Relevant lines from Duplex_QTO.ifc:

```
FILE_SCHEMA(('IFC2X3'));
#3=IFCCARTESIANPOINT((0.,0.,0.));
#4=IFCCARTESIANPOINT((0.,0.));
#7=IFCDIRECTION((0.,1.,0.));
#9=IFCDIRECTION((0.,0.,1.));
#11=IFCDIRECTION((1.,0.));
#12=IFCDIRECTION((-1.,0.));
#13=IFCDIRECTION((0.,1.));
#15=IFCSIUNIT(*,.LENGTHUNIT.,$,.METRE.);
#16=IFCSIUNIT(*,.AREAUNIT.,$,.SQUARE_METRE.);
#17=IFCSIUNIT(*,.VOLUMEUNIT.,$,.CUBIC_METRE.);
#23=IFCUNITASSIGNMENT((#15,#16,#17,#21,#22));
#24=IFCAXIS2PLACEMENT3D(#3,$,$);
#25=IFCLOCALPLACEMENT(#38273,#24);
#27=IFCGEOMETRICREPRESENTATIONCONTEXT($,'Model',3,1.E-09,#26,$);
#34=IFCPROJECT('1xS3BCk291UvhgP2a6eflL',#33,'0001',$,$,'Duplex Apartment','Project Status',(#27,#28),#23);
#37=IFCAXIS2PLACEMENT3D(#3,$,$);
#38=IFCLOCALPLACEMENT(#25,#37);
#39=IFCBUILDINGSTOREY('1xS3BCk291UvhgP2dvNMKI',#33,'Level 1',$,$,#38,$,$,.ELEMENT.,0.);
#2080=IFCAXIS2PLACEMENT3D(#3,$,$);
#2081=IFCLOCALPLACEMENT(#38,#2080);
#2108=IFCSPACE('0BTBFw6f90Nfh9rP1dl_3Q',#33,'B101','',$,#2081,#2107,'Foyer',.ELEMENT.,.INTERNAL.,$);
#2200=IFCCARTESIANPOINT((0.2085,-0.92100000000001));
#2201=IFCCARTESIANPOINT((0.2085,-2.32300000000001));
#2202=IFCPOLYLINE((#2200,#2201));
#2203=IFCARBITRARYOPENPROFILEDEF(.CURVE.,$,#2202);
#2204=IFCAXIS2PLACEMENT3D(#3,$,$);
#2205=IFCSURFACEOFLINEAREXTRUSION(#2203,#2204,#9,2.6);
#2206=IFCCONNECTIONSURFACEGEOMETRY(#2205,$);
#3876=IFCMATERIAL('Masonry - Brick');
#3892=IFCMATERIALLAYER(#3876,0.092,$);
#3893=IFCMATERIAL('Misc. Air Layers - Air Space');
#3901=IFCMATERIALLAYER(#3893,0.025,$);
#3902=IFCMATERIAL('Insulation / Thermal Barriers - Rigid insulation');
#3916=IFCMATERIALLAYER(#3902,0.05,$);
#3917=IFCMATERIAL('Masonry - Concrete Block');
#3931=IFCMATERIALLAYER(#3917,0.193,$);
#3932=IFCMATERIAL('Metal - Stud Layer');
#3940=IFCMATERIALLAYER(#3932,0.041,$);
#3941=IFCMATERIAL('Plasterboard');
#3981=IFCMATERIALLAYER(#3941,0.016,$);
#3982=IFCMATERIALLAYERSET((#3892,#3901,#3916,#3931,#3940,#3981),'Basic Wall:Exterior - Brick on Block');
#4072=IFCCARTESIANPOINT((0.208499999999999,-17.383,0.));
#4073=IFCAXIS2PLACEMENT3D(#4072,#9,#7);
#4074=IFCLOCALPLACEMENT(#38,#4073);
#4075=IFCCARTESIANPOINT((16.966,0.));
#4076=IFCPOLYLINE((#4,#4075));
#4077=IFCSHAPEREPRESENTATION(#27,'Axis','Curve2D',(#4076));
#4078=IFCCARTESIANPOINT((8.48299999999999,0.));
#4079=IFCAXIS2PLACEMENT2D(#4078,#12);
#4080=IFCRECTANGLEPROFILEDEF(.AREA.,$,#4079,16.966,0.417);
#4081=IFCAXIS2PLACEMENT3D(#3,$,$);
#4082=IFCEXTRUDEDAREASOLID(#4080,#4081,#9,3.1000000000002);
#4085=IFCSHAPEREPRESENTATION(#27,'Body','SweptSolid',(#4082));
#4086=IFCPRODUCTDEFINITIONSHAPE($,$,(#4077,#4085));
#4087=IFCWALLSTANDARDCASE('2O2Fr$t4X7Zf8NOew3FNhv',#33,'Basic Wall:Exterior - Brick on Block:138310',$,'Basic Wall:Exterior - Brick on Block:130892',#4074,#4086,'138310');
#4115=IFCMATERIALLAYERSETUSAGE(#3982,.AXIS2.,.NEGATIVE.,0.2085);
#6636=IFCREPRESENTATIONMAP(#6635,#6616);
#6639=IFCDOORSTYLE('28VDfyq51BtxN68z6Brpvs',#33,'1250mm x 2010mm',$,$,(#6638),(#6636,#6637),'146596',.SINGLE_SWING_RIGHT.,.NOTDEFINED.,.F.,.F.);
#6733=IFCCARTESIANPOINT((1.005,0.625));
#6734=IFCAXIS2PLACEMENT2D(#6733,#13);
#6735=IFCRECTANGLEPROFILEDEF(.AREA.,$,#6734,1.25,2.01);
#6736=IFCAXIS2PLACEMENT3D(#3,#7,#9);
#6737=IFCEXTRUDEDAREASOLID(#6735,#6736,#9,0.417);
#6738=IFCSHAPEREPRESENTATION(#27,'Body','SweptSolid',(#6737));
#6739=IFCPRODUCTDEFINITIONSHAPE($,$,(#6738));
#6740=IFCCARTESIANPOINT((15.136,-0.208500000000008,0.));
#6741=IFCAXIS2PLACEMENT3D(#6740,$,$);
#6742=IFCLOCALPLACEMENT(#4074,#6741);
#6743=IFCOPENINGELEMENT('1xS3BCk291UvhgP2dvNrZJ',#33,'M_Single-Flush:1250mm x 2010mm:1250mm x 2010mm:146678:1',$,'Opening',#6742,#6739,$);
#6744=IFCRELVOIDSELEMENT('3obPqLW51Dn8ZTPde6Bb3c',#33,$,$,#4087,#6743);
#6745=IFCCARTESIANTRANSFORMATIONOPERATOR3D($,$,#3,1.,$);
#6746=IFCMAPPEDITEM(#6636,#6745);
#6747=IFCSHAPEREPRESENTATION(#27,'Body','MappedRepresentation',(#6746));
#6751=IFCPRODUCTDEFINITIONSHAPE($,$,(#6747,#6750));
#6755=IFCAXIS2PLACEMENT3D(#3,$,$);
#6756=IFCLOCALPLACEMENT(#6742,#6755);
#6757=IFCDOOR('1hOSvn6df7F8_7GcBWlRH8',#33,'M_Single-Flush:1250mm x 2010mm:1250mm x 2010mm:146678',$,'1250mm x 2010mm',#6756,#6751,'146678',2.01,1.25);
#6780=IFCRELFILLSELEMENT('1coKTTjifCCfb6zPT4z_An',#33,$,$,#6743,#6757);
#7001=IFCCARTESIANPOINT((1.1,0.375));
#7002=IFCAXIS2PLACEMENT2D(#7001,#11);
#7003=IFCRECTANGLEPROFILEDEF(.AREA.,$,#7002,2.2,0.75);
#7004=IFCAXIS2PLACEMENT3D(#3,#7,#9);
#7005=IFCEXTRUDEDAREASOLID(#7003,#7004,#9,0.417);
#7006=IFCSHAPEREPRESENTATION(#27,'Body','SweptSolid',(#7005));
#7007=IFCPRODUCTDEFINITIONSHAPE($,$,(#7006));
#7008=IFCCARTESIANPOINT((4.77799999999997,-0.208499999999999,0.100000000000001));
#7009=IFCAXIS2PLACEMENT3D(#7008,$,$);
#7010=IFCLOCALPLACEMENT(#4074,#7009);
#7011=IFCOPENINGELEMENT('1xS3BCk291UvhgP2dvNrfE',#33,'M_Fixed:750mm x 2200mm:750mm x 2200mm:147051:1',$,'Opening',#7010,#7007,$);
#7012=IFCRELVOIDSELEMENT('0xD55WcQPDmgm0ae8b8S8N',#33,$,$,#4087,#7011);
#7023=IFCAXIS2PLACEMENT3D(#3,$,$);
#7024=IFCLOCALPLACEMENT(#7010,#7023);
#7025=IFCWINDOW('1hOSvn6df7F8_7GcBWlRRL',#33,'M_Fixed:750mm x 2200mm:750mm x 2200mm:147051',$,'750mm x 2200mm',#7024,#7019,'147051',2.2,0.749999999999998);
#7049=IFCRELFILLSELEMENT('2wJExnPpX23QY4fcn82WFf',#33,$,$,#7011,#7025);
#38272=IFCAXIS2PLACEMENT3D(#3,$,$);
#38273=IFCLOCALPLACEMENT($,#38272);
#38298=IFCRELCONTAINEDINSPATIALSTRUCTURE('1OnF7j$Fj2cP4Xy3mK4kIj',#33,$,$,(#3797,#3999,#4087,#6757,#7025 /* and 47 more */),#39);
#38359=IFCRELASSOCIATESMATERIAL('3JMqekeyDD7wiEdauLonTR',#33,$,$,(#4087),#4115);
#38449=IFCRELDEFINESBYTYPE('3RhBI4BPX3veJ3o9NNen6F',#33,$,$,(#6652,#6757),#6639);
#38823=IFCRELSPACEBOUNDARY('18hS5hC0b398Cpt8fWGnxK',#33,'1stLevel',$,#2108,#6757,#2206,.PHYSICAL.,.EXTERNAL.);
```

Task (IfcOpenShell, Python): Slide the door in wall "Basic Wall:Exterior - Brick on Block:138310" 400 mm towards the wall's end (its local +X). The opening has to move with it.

```python
import numpy as np
import ifcopenshell
import ifcopenshell.api.geometry
import ifcopenshell.util.placement
import ifcopenshell.util.unit

model = ifcopenshell.open("Duplex_QTO.ifc")
unit_scale = ifcopenshell.util.unit.calculate_unit_scale(model)

door = model.by_guid("1hOSvn6df7F8_7GcBWlRH8")
opening = door.FillsVoids[0].RelatingOpeningElement
wall = opening.VoidsElements[0].RelatingBuildingElement

wall_matrix = ifcopenshell.util.placement.get_local_placement(wall.ObjectPlacement)
shift = wall_matrix[:3, 0] * 0.4 / unit_scale
before = ifcopenshell.util.placement.get_local_placement(door.ObjectPlacement)[:3, 3].copy()

# The door is placed relative to its opening, so it follows when the opening moves.
matrix = ifcopenshell.util.placement.get_local_placement(opening.ObjectPlacement)
matrix[:3, 3] += shift
ifcopenshell.api.geometry.edit_object_placement(
    model, product=opening, matrix=matrix, is_si=False, should_transform_children=True
)

# Space boundary surfaces are stored in each space's coordinates; move them too.
for rel in door.ProvidesBoundaries:
    if not rel.ConnectionGeometry:
        continue
    surface = rel.ConnectionGeometry.SurfaceOnRelatingElement
    space_matrix = ifcopenshell.util.placement.get_local_placement(rel.RelatingSpace.ObjectPlacement)
    point = np.array(surface.Position.Location.Coordinates) + space_matrix[:3, :3].T @ shift
    surface.Position = model.createIfcAxis2Placement3D(
        model.createIfcCartesianPoint(point.tolist()), surface.Position.Axis, surface.Position.RefDirection
    )

after = ifcopenshell.util.placement.get_local_placement(door.ObjectPlacement)[:3, 3]
print("door moved by", (after - before).round(3) + 0.0)

model.write("Duplex_QTO_v2.ifc")
```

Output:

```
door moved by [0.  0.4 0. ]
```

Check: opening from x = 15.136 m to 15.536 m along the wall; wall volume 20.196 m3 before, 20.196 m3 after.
